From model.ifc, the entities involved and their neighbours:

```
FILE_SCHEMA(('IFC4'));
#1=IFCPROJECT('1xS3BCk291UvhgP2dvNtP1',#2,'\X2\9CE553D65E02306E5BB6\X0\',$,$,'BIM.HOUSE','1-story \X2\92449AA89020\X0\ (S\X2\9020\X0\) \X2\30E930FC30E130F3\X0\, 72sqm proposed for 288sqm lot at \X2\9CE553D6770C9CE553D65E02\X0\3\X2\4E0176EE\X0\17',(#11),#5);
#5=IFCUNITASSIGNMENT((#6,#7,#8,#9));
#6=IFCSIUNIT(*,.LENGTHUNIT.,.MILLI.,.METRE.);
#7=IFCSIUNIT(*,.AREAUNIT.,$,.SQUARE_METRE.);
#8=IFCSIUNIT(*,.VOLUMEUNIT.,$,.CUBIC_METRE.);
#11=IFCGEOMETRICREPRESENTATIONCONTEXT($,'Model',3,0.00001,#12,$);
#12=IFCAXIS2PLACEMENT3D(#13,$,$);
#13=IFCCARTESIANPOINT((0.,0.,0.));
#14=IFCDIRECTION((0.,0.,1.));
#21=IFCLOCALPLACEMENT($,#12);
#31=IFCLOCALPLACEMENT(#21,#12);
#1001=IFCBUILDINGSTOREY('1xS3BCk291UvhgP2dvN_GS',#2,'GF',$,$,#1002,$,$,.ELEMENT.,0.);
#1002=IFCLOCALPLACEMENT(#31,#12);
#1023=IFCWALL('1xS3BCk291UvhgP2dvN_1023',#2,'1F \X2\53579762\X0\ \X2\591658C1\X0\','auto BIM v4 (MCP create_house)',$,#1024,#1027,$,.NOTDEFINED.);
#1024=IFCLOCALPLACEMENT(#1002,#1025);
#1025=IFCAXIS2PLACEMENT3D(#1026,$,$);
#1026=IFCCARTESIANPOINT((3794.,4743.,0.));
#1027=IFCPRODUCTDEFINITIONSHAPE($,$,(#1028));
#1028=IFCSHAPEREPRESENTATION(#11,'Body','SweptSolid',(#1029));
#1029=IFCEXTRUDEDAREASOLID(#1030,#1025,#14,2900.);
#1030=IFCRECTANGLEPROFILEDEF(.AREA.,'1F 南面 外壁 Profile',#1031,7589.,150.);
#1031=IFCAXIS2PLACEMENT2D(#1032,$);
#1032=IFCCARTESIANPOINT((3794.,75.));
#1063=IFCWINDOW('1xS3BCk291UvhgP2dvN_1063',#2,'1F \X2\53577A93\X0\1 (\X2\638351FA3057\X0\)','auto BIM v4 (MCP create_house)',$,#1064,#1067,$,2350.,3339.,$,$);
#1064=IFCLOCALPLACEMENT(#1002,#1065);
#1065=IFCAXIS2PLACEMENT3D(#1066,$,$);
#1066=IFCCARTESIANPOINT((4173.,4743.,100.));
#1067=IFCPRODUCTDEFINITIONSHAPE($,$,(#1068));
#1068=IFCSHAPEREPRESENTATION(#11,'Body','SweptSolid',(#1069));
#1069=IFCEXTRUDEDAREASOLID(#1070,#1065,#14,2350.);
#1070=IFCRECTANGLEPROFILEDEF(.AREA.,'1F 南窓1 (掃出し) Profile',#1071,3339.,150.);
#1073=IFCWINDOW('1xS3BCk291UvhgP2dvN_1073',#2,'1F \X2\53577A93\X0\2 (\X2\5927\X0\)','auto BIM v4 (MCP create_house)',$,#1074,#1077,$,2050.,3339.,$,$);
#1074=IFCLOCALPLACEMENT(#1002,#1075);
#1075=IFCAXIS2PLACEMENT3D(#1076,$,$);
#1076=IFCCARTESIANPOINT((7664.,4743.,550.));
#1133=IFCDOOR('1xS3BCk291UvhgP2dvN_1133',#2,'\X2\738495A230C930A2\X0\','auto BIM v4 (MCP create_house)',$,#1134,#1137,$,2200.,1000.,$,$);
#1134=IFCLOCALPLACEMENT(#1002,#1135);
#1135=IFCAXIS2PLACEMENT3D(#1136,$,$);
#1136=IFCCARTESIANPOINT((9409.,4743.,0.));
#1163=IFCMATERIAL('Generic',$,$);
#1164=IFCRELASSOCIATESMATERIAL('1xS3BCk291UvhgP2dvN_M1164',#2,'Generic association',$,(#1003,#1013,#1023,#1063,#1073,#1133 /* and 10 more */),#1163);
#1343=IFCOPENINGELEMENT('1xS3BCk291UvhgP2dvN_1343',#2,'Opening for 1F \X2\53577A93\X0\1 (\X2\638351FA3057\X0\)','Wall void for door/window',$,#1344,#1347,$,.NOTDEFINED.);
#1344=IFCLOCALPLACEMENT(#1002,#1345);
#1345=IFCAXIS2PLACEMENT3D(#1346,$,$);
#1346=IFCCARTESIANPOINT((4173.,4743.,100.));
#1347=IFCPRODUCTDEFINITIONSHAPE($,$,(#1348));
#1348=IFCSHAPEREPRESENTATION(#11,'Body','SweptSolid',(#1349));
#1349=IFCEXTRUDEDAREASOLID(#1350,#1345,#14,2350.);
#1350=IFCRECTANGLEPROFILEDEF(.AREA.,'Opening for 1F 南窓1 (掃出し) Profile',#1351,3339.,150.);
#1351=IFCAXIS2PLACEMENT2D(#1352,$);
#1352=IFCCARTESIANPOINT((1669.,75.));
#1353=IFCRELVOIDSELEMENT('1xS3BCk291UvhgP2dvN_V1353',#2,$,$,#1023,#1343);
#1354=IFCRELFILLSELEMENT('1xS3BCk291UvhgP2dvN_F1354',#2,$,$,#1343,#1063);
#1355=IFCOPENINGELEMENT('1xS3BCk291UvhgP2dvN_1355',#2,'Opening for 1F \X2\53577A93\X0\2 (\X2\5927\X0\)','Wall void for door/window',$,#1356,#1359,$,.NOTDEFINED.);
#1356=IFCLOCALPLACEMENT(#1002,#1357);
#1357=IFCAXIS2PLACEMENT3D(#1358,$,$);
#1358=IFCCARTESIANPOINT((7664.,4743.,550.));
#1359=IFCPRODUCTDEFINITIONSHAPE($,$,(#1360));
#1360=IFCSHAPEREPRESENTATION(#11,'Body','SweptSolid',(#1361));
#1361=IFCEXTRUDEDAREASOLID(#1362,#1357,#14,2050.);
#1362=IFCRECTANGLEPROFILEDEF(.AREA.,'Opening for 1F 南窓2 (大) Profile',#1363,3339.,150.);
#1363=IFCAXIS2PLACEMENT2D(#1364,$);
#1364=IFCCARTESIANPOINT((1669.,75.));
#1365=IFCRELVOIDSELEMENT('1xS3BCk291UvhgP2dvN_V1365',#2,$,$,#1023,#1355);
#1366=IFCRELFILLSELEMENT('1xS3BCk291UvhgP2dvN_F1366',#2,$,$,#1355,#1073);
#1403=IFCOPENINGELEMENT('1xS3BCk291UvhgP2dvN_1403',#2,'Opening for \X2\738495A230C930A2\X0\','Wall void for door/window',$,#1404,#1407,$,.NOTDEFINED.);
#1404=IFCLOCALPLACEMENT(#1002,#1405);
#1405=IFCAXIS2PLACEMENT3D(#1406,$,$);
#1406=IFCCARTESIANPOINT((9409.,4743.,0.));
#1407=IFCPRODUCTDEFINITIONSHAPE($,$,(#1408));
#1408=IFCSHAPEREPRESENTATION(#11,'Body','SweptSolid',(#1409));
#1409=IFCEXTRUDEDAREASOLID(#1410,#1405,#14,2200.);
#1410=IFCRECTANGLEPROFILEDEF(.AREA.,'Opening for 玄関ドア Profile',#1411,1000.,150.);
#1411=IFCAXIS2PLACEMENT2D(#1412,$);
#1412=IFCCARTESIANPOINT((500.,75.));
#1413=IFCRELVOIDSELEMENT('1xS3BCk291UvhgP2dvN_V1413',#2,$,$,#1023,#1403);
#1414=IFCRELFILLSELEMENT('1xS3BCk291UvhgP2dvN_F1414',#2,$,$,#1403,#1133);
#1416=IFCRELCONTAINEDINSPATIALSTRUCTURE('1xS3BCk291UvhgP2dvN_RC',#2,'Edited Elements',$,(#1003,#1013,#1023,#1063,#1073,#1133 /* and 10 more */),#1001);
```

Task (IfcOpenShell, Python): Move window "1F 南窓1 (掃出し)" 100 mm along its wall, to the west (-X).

```python
import ifcopenshell
import ifcopenshell.api.geometry
import ifcopenshell.util.placement
import ifcopenshell.util.unit

model = ifcopenshell.open("model.ifc")
unit_scale = ifcopenshell.util.unit.calculate_unit_scale(model)

window = model.by_guid("1xS3BCk291UvhgP2dvN_1063")
opening = window.FillsVoids[0].RelatingOpeningElement
wall = opening.VoidsElements[0].RelatingBuildingElement

wall_matrix = ifcopenshell.util.placement.get_local_placement(wall.ObjectPlacement)
shift = wall_matrix[:3, 0] * -0.1 / unit_scale
before = ifcopenshell.util.placement.get_local_placement(window.ObjectPlacement)[:3, 3].copy()

# The window is not placed relative to its opening, so move both.
for product in (opening, window):
    matrix = ifcopenshell.util.placement.get_local_placement(product.ObjectPlacement)
    matrix[:3, 3] += shift
    ifcopenshell.api.geometry.edit_object_placement(model, product=product, matrix=matrix, is_si=False)

after = ifcopenshell.util.placement.get_local_placement(window.ObjectPlacement)[:3, 3]
print("window moved by", (after - before).round(3) + 0.0)

model.write("model-out.ifc")
```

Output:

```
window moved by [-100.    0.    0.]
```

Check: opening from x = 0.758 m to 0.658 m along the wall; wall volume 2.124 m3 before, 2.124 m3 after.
